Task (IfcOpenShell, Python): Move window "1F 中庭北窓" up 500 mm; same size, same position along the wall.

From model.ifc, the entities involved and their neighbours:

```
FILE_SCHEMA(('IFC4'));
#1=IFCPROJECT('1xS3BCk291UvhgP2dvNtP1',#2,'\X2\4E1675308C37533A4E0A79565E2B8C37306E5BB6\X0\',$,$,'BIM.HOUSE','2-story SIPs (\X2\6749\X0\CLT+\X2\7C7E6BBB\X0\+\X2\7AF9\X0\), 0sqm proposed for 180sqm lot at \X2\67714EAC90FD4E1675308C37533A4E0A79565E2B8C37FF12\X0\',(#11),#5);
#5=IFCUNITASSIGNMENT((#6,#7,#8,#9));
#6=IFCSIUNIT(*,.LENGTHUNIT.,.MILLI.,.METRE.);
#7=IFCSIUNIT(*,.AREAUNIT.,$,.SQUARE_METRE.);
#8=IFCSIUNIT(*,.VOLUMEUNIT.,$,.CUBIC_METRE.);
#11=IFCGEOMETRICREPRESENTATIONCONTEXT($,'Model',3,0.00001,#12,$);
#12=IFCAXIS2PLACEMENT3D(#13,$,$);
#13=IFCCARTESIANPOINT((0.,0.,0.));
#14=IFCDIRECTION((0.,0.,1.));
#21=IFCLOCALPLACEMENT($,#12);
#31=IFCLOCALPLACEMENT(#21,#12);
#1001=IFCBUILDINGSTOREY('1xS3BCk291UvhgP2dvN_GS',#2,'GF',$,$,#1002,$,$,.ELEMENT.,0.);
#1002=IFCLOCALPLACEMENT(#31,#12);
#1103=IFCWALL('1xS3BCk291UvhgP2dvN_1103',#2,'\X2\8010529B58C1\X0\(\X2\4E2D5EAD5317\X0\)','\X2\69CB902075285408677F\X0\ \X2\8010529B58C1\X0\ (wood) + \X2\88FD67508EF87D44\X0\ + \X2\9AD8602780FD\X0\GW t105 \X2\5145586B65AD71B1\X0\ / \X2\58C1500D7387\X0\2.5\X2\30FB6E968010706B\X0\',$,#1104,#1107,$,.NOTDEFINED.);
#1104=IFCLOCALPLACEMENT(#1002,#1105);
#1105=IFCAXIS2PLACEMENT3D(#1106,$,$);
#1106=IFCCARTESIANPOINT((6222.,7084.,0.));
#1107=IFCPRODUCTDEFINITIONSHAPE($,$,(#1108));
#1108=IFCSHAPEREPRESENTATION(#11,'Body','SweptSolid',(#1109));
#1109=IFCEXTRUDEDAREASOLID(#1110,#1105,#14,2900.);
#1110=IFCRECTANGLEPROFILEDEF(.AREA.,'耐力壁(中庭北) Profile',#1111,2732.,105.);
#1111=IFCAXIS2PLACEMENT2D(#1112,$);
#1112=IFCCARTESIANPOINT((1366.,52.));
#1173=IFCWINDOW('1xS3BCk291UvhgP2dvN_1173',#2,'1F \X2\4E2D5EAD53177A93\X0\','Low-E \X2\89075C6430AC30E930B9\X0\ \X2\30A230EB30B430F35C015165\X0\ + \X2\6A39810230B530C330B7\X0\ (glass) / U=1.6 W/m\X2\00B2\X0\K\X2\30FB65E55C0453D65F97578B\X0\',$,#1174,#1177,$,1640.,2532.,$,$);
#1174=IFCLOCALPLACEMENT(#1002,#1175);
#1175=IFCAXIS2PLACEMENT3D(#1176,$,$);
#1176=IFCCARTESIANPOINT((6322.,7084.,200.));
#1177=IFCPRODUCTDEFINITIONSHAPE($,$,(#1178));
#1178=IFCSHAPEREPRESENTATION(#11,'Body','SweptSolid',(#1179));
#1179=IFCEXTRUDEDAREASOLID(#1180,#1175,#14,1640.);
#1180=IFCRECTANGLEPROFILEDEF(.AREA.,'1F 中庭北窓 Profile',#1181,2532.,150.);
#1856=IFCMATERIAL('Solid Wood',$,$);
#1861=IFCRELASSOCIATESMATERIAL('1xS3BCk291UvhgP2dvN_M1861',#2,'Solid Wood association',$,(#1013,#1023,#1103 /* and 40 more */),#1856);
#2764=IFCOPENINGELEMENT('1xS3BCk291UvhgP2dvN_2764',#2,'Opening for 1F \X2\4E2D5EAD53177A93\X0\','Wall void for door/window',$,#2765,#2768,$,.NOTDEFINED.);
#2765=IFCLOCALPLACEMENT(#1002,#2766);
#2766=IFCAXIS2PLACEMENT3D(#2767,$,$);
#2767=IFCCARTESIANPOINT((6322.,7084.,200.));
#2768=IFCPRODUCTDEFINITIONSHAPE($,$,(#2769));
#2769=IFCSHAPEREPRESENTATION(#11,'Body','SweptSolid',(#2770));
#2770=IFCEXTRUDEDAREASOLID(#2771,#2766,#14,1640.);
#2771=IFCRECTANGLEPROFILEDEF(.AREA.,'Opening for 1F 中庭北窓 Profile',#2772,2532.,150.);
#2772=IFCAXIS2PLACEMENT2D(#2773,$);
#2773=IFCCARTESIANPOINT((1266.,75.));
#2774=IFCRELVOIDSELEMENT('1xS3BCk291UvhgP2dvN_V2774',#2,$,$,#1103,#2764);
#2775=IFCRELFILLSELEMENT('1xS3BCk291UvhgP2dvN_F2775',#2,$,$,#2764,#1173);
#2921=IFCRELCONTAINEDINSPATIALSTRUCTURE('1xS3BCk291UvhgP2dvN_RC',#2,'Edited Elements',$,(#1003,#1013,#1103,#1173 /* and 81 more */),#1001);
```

```python
import numpy as np
import ifcopenshell
import ifcopenshell.api.geometry
import ifcopenshell.util.placement
import ifcopenshell.util.unit

model = ifcopenshell.open("model.ifc")
unit_scale = ifcopenshell.util.unit.calculate_unit_scale(model)

window = model.by_guid("1xS3BCk291UvhgP2dvN_1173")
opening = window.FillsVoids[0].RelatingOpeningElement
dz = 0.5 / unit_scale

shift = np.array([0.0, 0.0, dz])
# The window is not placed relative to its opening, so move both.
for product in (opening, window):
    matrix = ifcopenshell.util.placement.get_local_placement(product.ObjectPlacement)
    matrix[:3, 3] += shift
    ifcopenshell.api.geometry.edit_object_placement(model, product=product, matrix=matrix, is_si=False)

print(f"moved by {dz * unit_scale:+.3f} m")

model.write("model_rev.ifc")
```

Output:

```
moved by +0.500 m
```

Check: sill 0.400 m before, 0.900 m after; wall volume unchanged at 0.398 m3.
